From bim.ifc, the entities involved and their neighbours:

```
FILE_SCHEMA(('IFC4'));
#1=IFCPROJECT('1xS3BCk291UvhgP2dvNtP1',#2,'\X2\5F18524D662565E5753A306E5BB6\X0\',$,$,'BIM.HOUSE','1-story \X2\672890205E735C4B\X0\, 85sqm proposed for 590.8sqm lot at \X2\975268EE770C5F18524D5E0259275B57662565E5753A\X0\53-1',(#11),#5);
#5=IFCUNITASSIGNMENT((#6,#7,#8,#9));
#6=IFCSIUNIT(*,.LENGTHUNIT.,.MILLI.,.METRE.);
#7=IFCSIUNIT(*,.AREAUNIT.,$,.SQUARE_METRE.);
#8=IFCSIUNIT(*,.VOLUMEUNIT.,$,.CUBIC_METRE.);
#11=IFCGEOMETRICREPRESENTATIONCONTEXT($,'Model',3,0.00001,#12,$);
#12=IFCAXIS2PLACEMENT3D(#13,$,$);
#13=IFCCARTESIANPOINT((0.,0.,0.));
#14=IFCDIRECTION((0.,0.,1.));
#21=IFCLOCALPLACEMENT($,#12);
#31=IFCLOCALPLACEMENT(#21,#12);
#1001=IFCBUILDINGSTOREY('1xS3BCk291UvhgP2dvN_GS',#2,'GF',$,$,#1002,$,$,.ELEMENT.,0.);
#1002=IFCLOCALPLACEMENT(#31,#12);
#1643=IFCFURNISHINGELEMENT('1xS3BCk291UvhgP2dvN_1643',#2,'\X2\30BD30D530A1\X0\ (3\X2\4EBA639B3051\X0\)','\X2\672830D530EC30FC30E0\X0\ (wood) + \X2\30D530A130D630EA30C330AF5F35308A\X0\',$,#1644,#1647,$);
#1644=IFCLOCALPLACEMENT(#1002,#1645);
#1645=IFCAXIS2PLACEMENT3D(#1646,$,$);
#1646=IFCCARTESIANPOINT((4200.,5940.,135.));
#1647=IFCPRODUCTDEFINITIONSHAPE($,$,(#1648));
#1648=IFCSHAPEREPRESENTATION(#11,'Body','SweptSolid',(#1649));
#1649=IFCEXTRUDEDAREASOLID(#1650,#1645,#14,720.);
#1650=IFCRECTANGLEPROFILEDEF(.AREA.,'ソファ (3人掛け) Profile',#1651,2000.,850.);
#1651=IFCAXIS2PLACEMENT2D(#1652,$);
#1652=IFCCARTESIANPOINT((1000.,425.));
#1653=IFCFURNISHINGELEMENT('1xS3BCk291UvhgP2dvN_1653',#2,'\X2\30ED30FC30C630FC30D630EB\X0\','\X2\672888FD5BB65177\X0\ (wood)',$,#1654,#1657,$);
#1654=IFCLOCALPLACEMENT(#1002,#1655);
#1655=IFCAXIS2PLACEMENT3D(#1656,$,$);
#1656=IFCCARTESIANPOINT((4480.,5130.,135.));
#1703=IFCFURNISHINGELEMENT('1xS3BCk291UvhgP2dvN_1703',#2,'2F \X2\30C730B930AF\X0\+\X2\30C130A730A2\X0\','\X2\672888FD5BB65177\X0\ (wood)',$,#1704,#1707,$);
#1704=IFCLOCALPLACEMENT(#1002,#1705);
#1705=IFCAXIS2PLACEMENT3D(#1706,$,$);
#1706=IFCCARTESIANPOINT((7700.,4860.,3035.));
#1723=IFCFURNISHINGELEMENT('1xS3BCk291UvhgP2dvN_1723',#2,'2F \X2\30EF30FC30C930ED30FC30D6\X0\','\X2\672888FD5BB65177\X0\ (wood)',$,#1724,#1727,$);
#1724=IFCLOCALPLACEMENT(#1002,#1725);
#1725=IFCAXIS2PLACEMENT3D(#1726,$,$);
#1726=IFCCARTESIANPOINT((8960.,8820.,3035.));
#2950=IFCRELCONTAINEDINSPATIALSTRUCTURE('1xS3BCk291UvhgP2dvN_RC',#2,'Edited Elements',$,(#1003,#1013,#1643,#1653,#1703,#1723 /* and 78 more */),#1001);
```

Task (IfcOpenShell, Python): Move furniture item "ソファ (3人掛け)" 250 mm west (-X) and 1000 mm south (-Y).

```python
import ifcopenshell
import ifcopenshell.api.geometry
import ifcopenshell.util.placement
import ifcopenshell.util.unit

model = ifcopenshell.open("bim.ifc")
unit_scale = ifcopenshell.util.unit.calculate_unit_scale(model)

item = model.by_guid("1xS3BCk291UvhgP2dvN_1643")
matrix = ifcopenshell.util.placement.get_local_placement(item.ObjectPlacement)
matrix[0, 3] -= 0.25 / unit_scale
matrix[1, 3] -= 1 / unit_scale
ifcopenshell.api.geometry.edit_object_placement(model, product=item, matrix=matrix, is_si=False)

print(ifcopenshell.util.placement.get_local_placement(item.ObjectPlacement).round(3) + 0.0)

model.write("bim-out.ifc")
```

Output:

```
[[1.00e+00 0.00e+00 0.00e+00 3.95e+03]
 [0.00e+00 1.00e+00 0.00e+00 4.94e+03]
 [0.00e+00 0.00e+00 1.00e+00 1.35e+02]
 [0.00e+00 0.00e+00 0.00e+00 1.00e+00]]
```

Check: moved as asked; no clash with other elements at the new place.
